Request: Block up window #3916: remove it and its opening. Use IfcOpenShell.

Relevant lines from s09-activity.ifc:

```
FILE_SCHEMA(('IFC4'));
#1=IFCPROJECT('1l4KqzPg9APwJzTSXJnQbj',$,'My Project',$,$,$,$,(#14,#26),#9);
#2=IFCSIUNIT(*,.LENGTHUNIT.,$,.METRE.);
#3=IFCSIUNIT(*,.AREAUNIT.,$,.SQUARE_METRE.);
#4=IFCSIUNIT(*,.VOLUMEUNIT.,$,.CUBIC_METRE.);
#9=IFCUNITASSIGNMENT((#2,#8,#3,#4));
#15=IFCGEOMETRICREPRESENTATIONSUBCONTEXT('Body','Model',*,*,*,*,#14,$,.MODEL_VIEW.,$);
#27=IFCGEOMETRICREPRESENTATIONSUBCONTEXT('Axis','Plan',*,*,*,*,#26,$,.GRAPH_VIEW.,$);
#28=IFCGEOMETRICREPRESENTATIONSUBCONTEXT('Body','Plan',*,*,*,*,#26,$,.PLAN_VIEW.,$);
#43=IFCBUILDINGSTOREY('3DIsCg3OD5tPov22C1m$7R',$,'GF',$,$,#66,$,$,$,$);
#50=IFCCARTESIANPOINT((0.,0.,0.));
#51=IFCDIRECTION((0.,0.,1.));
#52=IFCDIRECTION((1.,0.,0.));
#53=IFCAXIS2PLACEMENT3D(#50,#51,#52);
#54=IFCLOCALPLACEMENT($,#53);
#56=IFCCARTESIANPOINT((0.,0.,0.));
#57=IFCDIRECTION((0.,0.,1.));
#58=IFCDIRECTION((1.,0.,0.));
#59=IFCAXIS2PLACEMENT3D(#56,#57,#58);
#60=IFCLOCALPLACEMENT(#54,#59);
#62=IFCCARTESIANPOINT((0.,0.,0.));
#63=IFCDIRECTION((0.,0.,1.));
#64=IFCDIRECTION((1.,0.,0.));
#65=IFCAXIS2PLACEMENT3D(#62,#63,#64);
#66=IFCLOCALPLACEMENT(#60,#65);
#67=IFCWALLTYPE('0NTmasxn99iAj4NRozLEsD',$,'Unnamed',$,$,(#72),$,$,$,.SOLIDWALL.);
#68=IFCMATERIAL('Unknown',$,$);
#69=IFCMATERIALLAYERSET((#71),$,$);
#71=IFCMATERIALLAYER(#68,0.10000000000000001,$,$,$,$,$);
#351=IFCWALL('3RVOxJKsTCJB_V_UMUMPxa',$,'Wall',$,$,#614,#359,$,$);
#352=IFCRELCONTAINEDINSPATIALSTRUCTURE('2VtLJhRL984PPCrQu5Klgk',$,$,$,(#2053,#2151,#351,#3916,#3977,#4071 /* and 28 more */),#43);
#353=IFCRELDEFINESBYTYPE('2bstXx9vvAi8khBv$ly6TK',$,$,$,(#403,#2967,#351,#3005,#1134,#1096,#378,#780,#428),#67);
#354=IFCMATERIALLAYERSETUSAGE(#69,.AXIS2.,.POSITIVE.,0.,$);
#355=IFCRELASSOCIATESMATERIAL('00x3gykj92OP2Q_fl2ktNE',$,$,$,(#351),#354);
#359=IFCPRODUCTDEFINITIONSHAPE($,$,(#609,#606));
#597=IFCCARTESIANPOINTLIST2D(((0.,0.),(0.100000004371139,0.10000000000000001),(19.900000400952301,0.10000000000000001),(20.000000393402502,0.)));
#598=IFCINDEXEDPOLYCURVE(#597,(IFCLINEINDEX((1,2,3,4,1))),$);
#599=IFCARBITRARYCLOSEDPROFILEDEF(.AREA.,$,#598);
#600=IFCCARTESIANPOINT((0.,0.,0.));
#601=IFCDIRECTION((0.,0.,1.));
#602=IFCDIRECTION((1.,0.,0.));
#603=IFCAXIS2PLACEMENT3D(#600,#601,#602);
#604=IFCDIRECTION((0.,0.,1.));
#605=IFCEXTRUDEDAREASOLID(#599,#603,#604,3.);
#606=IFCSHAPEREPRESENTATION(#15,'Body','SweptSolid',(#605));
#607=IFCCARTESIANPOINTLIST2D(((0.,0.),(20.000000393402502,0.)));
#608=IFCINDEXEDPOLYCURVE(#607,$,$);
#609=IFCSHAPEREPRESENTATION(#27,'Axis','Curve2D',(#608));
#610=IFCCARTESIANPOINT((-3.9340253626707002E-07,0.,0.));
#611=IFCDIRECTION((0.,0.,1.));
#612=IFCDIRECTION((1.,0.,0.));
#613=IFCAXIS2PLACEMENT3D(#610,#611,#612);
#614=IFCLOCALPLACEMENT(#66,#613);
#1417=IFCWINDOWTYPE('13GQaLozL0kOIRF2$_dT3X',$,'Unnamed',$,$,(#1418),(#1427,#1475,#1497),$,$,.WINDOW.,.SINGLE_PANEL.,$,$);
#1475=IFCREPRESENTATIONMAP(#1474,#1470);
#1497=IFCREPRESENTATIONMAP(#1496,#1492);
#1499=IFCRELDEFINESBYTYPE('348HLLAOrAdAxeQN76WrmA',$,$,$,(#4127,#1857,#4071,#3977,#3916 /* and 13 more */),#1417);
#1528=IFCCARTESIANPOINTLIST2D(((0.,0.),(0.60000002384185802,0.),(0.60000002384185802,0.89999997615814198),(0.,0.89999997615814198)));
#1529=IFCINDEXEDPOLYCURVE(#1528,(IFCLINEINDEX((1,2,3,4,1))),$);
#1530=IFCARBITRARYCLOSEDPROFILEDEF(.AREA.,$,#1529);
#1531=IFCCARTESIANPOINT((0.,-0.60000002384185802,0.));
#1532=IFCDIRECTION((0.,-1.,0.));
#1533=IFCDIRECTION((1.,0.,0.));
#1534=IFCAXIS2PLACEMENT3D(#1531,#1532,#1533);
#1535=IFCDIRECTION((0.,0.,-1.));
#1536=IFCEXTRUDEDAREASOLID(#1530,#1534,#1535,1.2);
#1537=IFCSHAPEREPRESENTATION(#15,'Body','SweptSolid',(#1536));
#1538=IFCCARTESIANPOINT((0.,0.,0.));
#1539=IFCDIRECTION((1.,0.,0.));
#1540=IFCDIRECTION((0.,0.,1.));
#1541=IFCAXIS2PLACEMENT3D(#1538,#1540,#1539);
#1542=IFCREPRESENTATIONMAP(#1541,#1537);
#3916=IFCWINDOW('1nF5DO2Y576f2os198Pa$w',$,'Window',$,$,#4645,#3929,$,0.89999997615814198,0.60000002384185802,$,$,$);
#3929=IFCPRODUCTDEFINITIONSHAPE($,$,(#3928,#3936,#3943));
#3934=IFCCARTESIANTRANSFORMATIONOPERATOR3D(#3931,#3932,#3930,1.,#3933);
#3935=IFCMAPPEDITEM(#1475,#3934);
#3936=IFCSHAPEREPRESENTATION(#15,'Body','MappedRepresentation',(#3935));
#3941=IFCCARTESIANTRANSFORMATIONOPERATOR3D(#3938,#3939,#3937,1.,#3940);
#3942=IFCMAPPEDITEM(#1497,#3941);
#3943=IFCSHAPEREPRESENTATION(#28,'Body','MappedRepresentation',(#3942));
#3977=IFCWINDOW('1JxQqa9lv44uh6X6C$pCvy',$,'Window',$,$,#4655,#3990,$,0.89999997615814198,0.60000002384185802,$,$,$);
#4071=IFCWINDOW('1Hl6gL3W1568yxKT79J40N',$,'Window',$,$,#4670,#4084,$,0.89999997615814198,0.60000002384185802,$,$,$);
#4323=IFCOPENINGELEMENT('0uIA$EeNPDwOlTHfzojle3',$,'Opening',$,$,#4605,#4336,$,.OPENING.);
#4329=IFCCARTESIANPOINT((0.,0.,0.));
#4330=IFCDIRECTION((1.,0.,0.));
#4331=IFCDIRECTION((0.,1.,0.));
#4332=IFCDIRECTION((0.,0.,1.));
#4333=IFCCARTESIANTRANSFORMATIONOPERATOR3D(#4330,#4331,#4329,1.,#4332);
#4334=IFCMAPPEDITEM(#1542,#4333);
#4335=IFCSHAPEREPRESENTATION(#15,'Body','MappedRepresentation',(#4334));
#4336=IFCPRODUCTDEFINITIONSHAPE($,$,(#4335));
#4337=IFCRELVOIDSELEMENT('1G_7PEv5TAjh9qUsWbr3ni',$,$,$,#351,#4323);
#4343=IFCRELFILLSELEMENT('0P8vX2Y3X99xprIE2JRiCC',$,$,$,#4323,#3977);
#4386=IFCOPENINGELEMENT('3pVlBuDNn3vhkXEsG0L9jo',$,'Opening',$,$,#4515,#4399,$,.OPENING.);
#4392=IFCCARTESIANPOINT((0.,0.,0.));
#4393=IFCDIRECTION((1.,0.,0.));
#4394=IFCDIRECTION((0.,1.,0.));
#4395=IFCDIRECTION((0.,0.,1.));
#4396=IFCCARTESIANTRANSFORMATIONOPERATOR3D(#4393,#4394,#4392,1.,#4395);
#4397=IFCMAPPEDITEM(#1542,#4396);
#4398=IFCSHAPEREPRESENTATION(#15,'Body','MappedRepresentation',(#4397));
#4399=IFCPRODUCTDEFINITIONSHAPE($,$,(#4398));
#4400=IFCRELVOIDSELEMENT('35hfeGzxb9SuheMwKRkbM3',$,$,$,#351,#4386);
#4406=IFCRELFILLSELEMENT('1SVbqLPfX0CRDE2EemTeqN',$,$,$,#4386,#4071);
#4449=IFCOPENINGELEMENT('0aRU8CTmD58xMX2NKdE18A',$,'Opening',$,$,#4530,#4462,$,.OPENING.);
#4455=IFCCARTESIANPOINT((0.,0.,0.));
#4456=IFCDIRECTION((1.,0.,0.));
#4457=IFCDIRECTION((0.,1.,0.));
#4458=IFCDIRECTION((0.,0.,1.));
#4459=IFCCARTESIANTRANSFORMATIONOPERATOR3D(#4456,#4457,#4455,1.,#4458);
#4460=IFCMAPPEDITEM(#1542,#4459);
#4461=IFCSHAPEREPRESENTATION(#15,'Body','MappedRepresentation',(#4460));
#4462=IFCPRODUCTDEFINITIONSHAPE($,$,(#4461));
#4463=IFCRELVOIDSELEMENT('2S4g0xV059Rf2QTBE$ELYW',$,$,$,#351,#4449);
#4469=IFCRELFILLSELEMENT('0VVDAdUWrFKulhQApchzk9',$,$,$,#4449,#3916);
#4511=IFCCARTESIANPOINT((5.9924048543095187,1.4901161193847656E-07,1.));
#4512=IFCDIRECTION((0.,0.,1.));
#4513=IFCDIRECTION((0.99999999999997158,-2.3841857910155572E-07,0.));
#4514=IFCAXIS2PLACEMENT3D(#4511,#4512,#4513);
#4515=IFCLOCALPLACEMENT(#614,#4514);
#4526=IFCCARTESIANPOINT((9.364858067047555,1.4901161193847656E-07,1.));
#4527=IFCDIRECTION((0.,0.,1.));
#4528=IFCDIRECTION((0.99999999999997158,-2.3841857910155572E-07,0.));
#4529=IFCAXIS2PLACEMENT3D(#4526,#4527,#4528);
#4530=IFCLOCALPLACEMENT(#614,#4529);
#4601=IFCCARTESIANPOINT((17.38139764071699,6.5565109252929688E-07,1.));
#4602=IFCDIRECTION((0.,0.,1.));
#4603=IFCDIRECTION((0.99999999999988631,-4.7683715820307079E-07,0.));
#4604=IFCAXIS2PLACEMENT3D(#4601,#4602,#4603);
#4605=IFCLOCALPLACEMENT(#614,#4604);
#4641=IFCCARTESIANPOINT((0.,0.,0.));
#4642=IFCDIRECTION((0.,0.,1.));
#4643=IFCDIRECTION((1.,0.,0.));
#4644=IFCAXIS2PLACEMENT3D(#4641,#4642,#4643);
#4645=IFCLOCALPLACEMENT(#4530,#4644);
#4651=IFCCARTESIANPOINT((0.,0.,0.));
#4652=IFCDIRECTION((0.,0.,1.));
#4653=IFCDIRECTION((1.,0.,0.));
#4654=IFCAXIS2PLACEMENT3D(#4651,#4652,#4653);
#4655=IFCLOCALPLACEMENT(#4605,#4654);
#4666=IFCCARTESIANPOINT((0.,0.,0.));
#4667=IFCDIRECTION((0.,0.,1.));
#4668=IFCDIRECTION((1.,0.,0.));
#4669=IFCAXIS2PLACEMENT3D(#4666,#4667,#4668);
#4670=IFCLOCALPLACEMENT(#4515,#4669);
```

```python
import ifcopenshell
import ifcopenshell.api.feature
import ifcopenshell.api.root
import ifcopenshell.geom
import ifcopenshell.util.shape

model = ifcopenshell.open("s09-activity.ifc")
settings = ifcopenshell.geom.settings()


def volume(element):
    """Net volume in cubic metres, openings subtracted."""
    shape = ifcopenshell.geom.create_shape(settings, element)
    return ifcopenshell.util.shape.get_volume(shape.geometry)


window = model.by_id(3916)
opening = window.FillsVoids[0].RelatingOpeningElement
wall = opening.VoidsElements[0].RelatingBuildingElement
before = volume(wall)

ifcopenshell.api.root.remove_product(model, product=window)
ifcopenshell.api.feature.remove_feature(model, feature=opening)

after = volume(wall)

print(f"wall volume {before:.3f} -> {after:.3f} m3")

model.write("s09-activity_updated.ifc")
```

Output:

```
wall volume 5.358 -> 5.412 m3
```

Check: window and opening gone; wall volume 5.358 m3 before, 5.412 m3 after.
